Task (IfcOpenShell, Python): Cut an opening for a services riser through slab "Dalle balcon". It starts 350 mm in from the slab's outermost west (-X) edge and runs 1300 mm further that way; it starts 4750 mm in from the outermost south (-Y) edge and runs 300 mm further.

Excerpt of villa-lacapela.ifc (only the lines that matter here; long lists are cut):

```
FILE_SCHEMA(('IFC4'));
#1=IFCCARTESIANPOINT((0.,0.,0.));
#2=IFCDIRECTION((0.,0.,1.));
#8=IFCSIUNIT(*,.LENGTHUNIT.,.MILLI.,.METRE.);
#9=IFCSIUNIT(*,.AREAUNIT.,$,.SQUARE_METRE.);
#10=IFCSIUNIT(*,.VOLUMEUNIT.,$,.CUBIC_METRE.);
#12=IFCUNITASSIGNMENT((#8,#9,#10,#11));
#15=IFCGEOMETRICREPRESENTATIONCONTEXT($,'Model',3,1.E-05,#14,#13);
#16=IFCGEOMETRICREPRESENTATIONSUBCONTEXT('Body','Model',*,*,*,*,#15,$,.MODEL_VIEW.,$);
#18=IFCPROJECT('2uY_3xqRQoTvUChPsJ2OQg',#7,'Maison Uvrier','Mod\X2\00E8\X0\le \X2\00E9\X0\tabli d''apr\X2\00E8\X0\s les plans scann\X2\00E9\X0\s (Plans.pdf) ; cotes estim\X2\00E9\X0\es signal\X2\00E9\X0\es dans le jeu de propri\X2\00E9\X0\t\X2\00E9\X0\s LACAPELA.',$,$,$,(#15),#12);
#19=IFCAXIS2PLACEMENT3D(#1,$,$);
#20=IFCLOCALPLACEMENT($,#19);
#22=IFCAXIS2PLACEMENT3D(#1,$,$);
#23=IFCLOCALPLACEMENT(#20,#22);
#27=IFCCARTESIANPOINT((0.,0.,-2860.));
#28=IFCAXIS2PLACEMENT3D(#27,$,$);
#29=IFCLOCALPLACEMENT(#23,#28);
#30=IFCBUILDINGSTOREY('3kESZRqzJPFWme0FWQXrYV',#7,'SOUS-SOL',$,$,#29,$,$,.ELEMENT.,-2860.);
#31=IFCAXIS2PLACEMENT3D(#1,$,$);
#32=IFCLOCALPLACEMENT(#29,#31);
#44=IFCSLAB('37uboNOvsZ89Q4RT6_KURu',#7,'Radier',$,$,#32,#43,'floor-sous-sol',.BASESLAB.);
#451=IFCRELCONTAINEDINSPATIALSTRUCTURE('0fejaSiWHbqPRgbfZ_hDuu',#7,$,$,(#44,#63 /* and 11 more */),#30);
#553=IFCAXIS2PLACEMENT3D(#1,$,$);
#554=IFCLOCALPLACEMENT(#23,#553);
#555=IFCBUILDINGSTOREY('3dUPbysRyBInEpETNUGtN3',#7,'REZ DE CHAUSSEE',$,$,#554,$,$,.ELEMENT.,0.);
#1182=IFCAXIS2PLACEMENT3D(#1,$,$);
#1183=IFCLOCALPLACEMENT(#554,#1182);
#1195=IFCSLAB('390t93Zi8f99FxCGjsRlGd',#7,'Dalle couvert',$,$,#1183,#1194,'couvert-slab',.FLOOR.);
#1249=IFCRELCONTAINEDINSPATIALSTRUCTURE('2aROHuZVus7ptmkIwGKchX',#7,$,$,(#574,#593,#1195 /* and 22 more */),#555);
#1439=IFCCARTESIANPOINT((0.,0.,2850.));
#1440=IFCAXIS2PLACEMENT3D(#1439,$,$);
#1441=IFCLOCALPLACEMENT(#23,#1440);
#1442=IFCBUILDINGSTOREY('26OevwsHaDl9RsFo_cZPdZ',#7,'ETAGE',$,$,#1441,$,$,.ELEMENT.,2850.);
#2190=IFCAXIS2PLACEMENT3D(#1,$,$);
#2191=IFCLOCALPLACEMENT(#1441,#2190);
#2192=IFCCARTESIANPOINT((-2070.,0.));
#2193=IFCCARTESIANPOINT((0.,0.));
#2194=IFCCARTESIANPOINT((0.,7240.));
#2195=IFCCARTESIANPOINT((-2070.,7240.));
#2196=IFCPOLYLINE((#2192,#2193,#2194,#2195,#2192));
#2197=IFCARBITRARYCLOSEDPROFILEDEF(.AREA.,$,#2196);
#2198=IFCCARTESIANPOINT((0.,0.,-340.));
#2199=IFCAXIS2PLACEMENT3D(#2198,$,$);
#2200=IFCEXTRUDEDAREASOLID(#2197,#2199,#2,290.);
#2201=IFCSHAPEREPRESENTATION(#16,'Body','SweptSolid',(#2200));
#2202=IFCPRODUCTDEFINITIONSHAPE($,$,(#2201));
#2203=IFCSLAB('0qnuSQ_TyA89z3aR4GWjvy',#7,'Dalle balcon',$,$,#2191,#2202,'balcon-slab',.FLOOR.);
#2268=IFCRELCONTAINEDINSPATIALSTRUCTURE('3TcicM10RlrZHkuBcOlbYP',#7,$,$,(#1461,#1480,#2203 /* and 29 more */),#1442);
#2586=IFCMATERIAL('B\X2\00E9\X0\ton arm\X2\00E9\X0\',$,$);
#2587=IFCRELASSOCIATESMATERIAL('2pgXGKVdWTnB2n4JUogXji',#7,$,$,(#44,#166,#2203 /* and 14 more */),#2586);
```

```python
import numpy as np
import ifcopenshell
import ifcopenshell.api.feature
import ifcopenshell.api.geometry
import ifcopenshell.api.root
import ifcopenshell.geom
import ifcopenshell.util.placement
import ifcopenshell.util.representation
import ifcopenshell.util.shape
import ifcopenshell.util.unit

model = ifcopenshell.open("villa-lacapela.ifc")
unit_scale = ifcopenshell.util.unit.calculate_unit_scale(model)
settings = ifcopenshell.geom.settings()


def volume(element):
    """Net volume in cubic metres, openings subtracted."""
    shape = ifcopenshell.geom.create_shape(settings, element)
    return ifcopenshell.util.shape.get_volume(shape.geometry)


slab = model.by_guid("0qnuSQ_TyA89z3aR4GWjvy")
before = volume(slab)

# Extent in the slab's own axes, in metres. The edges named are its -X and -Y sides.
slab_shape = ifcopenshell.geom.create_shape(settings, slab)
vertices = ifcopenshell.util.shape.get_vertices(slab_shape.geometry)
x_min, y_min, bottom = vertices.min(axis=0)
top = vertices[:, 2].max()

opening = ifcopenshell.api.root.create_entity(model, ifc_class="IfcOpeningElement", name="Services riser opening", predefined_type="OPENING")
context = ifcopenshell.util.representation.get_context(model, "Model", "Body", "MODEL_VIEW")
width, depth = 1.3, 0.3
outline = [(0.0, 0.0), (width, 0.0), (width, depth), (0.0, depth), (0.0, 0.0)]
# Overshoot both faces by 50 mm so the cut is clean.
shape = ifcopenshell.api.geometry.add_slab_representation(
    model, context=context, depth=top - bottom + 0.1, polyline=outline
)
ifcopenshell.api.geometry.assign_representation(model, product=opening, representation=shape)

matrix = ifcopenshell.util.placement.get_local_placement(slab.ObjectPlacement)
matrix[:, 3] = matrix @ np.append(np.array([x_min + 0.35, y_min + 4.75, bottom - 0.05]) / unit_scale, 1.0)
ifcopenshell.api.geometry.edit_object_placement(model, product=opening, matrix=matrix, is_si=False)
ifcopenshell.api.feature.add_feature(model, feature=opening, element=slab)

after = volume(slab)

print(f"slab volume {before:.3f} -> {after:.3f} m3")

model.write("villa-lacapela_updated.ifc")
```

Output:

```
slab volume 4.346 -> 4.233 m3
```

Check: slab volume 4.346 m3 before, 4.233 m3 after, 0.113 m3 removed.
